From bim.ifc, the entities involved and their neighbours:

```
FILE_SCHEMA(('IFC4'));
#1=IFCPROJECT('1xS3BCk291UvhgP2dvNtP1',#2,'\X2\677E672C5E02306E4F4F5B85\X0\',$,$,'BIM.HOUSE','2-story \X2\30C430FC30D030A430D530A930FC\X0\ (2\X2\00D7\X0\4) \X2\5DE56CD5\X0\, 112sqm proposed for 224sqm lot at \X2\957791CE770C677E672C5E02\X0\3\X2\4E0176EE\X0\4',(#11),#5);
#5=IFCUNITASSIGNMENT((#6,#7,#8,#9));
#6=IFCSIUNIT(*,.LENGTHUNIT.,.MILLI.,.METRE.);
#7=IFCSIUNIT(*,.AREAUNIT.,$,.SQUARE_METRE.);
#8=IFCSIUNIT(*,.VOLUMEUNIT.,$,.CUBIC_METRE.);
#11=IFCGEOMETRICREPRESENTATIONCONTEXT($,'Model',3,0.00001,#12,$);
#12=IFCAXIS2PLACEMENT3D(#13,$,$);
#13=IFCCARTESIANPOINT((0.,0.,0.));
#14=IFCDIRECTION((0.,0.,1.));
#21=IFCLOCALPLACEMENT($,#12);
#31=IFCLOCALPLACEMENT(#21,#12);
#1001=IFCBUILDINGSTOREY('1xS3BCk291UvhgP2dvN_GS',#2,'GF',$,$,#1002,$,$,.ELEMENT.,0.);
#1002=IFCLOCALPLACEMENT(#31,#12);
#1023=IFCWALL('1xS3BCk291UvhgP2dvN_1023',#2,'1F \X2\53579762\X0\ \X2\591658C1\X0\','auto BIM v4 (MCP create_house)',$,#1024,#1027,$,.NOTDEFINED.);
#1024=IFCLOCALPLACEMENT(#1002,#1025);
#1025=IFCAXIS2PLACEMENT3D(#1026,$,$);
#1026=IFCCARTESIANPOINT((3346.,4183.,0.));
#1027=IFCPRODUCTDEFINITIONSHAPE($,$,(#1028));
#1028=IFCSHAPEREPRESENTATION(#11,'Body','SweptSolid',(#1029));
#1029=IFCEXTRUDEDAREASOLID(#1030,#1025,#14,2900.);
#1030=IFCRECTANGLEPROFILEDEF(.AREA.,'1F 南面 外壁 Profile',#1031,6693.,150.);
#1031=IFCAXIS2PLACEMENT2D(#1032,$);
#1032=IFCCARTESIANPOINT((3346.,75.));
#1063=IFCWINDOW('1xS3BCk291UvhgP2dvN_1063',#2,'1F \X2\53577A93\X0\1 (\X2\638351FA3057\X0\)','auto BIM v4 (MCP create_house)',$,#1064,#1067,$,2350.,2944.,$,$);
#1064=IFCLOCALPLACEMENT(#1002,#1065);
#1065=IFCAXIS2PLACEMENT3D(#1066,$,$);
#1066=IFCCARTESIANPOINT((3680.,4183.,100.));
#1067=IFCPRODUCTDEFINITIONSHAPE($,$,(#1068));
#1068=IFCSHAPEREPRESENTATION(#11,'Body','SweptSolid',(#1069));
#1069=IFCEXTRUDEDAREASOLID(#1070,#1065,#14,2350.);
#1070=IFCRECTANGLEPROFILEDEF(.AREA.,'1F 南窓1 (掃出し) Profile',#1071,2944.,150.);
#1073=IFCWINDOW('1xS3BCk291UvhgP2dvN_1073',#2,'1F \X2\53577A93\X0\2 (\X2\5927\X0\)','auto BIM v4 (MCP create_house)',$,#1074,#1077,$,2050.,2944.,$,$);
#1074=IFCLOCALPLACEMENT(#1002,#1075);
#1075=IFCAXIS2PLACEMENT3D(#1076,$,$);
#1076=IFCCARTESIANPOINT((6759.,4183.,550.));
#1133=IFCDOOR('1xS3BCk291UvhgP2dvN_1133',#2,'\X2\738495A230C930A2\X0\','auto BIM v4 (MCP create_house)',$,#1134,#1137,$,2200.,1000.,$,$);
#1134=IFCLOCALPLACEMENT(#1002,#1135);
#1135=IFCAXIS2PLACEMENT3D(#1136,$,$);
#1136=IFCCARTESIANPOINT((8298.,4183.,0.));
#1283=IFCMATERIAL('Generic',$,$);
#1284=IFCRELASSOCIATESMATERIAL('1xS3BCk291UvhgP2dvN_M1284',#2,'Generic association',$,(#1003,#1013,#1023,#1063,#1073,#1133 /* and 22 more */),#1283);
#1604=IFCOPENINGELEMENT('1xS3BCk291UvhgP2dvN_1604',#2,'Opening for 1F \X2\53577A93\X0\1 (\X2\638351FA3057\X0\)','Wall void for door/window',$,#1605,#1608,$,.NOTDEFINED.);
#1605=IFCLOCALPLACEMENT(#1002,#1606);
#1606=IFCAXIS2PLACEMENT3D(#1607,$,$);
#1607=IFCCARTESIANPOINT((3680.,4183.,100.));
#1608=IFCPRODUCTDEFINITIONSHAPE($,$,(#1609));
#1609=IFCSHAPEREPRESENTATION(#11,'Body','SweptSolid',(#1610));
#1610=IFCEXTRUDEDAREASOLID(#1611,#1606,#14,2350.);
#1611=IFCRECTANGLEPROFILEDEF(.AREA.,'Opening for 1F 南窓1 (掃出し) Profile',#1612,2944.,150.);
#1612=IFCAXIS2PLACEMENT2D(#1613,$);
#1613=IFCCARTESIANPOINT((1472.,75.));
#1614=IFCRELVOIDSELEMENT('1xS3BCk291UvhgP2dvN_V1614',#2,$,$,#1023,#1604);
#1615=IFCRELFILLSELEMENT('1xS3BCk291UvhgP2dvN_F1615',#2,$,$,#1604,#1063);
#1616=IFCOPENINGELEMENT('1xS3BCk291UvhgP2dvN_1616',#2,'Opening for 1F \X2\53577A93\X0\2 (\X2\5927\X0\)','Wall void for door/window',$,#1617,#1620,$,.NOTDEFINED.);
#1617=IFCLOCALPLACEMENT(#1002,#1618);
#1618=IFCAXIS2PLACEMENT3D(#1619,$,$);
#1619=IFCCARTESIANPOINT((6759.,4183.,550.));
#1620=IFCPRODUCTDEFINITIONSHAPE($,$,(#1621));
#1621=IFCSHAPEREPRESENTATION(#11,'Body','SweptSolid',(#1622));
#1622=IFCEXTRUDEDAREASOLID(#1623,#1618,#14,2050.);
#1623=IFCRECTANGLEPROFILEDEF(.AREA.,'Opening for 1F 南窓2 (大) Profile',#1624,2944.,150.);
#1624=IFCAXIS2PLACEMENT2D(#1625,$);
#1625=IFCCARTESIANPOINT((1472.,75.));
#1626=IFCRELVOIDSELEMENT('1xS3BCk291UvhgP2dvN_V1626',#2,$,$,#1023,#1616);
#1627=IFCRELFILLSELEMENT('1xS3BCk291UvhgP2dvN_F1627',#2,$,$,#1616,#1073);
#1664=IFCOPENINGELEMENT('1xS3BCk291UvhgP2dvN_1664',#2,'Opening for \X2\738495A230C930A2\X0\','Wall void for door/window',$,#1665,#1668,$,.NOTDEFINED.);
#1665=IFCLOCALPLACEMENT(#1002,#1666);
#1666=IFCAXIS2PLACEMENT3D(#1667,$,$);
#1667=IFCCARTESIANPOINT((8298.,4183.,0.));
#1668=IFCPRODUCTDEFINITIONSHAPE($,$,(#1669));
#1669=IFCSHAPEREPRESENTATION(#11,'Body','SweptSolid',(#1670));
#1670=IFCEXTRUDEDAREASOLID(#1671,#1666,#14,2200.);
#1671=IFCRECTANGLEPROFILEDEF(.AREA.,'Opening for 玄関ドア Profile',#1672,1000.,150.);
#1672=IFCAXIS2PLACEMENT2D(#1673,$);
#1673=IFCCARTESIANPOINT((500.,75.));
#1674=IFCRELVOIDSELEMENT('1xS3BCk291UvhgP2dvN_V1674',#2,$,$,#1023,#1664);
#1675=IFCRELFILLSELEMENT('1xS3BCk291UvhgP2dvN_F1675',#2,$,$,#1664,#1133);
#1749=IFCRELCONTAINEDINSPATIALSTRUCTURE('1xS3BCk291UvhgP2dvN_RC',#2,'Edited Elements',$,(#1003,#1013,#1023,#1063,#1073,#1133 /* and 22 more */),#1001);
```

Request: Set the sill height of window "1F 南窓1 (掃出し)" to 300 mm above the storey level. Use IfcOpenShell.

```python
import numpy as np
import ifcopenshell
import ifcopenshell.api.geometry
import ifcopenshell.geom
import ifcopenshell.util.element
import ifcopenshell.util.placement
import ifcopenshell.util.shape
import ifcopenshell.util.unit

model = ifcopenshell.open("bim.ifc")
unit_scale = ifcopenshell.util.unit.calculate_unit_scale(model)

window = model.by_id(1063)
opening = window.FillsVoids[0].RelatingOpeningElement
storey = ifcopenshell.util.element.get_container(window, ifc_class="IfcBuildingStorey")
level = ifcopenshell.util.placement.get_local_placement(storey.ObjectPlacement)[2, 3]

# The opening's origin need not be at the sill, so measure its lowest point.
shape = ifcopenshell.geom.create_shape(ifcopenshell.geom.settings(), opening)
bottom = ifcopenshell.util.shape.get_shape_bottom_elevation(shape, shape.geometry) / unit_scale
dz = level + 300.0 - bottom

shift = np.array([0.0, 0.0, dz])
# The window is not placed relative to its opening, so move both.
for product in (opening, window):
    matrix = ifcopenshell.util.placement.get_local_placement(product.ObjectPlacement)
    matrix[:3, 3] += shift
    ifcopenshell.api.geometry.edit_object_placement(model, product=product, matrix=matrix, is_si=False)

print(f"moved by {dz * unit_scale:+.3f} m")

model.write("bim_edited.ifc")
```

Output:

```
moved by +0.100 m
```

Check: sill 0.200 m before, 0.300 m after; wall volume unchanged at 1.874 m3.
